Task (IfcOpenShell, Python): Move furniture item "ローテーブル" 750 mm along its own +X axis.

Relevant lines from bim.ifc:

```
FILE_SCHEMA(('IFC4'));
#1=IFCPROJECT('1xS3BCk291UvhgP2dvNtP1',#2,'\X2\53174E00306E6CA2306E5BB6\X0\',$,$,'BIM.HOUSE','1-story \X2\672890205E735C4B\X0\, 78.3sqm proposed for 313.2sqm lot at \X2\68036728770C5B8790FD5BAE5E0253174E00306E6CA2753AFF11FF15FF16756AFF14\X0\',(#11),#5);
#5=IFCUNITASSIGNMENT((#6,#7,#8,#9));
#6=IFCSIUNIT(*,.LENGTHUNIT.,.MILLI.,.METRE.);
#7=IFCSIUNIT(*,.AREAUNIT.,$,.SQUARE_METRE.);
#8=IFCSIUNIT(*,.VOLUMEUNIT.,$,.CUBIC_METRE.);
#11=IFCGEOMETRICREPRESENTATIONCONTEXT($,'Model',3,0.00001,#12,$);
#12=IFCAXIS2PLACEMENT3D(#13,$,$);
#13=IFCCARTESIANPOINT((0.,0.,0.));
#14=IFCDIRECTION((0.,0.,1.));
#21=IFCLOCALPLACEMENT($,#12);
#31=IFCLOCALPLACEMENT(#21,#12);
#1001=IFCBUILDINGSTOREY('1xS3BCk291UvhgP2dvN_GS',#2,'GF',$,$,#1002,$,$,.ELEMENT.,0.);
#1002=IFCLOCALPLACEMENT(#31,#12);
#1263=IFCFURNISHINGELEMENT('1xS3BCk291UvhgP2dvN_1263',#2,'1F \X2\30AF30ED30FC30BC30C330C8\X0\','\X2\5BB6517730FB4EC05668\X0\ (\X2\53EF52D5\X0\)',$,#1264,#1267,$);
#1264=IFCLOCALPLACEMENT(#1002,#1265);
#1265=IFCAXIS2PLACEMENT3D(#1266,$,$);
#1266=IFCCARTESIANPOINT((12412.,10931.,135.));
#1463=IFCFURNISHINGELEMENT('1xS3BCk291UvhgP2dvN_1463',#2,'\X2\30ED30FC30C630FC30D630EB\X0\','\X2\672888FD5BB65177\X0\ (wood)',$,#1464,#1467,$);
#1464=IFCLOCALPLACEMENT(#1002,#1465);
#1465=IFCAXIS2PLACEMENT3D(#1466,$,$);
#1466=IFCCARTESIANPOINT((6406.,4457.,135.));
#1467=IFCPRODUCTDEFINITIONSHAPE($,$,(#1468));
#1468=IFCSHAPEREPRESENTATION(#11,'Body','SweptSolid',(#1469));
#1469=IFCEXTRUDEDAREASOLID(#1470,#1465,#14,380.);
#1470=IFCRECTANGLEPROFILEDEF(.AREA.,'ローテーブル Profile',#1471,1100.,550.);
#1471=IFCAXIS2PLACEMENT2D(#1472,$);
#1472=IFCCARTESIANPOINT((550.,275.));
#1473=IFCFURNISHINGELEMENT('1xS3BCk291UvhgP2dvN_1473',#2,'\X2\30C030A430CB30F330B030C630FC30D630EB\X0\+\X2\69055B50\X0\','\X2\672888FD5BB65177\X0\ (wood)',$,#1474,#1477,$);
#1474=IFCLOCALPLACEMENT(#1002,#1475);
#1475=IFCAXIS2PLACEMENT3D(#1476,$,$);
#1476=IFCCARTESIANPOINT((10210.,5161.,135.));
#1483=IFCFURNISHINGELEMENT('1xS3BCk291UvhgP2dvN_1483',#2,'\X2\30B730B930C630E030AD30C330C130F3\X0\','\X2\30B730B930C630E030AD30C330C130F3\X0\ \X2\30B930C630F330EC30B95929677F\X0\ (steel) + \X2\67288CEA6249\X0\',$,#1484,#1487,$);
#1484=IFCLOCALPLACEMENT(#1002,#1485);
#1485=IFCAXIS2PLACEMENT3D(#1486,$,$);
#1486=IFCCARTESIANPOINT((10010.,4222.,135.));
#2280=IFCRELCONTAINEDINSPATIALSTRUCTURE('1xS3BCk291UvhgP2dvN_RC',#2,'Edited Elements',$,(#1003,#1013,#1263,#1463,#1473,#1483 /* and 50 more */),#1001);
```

```python
import ifcopenshell
import ifcopenshell.api.geometry
import ifcopenshell.util.placement

model = ifcopenshell.open("bim.ifc")

item = model.by_id(1463)
matrix = ifcopenshell.util.placement.get_local_placement(item.ObjectPlacement)
matrix[:3, 3] += matrix[:3, 0] * 750.0
ifcopenshell.api.geometry.edit_object_placement(model, product=item, matrix=matrix, is_si=False)

print(ifcopenshell.util.placement.get_local_placement(item.ObjectPlacement).round(3) + 0.0)

model.write("bim_rev.ifc")
```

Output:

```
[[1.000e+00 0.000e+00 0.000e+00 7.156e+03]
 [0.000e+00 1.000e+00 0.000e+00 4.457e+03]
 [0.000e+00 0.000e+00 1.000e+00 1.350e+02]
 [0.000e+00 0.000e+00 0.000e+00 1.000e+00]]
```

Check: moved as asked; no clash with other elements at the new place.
